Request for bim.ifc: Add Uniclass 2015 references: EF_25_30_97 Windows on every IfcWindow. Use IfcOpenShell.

First a look at what the model holds.

```python
import ifcopenshell

model = ifcopenshell.open("bim.ifc")
print(model.schema)
print("classifications:", [c.Name for c in model.by_type("IfcClassification")])
for ifc_class in ("IfcDoor", "IfcRoof", "IfcStair", "IfcWall", "IfcWindow"):
    print(ifc_class, len(model.by_type(ifc_class)))
```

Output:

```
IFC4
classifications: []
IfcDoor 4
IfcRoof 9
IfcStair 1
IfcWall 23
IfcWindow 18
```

```python
import ifcopenshell
import ifcopenshell.api.classification

model = ifcopenshell.open("bim.ifc")

system = ifcopenshell.api.classification.add_classification(model, classification="Uniclass 2015")

codes = {
    "IfcWindow": ("EF_25_30_97", "Windows"),
}
for ifc_class, (code, name) in codes.items():
    products = model.by_type(ifc_class)
    ifcopenshell.api.classification.add_reference(
        model, products=products, classification=system, identification=code, name=name
    )
    print(code, len(products))

model.write("bim_rev.ifc")
```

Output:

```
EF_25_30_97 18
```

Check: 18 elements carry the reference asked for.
